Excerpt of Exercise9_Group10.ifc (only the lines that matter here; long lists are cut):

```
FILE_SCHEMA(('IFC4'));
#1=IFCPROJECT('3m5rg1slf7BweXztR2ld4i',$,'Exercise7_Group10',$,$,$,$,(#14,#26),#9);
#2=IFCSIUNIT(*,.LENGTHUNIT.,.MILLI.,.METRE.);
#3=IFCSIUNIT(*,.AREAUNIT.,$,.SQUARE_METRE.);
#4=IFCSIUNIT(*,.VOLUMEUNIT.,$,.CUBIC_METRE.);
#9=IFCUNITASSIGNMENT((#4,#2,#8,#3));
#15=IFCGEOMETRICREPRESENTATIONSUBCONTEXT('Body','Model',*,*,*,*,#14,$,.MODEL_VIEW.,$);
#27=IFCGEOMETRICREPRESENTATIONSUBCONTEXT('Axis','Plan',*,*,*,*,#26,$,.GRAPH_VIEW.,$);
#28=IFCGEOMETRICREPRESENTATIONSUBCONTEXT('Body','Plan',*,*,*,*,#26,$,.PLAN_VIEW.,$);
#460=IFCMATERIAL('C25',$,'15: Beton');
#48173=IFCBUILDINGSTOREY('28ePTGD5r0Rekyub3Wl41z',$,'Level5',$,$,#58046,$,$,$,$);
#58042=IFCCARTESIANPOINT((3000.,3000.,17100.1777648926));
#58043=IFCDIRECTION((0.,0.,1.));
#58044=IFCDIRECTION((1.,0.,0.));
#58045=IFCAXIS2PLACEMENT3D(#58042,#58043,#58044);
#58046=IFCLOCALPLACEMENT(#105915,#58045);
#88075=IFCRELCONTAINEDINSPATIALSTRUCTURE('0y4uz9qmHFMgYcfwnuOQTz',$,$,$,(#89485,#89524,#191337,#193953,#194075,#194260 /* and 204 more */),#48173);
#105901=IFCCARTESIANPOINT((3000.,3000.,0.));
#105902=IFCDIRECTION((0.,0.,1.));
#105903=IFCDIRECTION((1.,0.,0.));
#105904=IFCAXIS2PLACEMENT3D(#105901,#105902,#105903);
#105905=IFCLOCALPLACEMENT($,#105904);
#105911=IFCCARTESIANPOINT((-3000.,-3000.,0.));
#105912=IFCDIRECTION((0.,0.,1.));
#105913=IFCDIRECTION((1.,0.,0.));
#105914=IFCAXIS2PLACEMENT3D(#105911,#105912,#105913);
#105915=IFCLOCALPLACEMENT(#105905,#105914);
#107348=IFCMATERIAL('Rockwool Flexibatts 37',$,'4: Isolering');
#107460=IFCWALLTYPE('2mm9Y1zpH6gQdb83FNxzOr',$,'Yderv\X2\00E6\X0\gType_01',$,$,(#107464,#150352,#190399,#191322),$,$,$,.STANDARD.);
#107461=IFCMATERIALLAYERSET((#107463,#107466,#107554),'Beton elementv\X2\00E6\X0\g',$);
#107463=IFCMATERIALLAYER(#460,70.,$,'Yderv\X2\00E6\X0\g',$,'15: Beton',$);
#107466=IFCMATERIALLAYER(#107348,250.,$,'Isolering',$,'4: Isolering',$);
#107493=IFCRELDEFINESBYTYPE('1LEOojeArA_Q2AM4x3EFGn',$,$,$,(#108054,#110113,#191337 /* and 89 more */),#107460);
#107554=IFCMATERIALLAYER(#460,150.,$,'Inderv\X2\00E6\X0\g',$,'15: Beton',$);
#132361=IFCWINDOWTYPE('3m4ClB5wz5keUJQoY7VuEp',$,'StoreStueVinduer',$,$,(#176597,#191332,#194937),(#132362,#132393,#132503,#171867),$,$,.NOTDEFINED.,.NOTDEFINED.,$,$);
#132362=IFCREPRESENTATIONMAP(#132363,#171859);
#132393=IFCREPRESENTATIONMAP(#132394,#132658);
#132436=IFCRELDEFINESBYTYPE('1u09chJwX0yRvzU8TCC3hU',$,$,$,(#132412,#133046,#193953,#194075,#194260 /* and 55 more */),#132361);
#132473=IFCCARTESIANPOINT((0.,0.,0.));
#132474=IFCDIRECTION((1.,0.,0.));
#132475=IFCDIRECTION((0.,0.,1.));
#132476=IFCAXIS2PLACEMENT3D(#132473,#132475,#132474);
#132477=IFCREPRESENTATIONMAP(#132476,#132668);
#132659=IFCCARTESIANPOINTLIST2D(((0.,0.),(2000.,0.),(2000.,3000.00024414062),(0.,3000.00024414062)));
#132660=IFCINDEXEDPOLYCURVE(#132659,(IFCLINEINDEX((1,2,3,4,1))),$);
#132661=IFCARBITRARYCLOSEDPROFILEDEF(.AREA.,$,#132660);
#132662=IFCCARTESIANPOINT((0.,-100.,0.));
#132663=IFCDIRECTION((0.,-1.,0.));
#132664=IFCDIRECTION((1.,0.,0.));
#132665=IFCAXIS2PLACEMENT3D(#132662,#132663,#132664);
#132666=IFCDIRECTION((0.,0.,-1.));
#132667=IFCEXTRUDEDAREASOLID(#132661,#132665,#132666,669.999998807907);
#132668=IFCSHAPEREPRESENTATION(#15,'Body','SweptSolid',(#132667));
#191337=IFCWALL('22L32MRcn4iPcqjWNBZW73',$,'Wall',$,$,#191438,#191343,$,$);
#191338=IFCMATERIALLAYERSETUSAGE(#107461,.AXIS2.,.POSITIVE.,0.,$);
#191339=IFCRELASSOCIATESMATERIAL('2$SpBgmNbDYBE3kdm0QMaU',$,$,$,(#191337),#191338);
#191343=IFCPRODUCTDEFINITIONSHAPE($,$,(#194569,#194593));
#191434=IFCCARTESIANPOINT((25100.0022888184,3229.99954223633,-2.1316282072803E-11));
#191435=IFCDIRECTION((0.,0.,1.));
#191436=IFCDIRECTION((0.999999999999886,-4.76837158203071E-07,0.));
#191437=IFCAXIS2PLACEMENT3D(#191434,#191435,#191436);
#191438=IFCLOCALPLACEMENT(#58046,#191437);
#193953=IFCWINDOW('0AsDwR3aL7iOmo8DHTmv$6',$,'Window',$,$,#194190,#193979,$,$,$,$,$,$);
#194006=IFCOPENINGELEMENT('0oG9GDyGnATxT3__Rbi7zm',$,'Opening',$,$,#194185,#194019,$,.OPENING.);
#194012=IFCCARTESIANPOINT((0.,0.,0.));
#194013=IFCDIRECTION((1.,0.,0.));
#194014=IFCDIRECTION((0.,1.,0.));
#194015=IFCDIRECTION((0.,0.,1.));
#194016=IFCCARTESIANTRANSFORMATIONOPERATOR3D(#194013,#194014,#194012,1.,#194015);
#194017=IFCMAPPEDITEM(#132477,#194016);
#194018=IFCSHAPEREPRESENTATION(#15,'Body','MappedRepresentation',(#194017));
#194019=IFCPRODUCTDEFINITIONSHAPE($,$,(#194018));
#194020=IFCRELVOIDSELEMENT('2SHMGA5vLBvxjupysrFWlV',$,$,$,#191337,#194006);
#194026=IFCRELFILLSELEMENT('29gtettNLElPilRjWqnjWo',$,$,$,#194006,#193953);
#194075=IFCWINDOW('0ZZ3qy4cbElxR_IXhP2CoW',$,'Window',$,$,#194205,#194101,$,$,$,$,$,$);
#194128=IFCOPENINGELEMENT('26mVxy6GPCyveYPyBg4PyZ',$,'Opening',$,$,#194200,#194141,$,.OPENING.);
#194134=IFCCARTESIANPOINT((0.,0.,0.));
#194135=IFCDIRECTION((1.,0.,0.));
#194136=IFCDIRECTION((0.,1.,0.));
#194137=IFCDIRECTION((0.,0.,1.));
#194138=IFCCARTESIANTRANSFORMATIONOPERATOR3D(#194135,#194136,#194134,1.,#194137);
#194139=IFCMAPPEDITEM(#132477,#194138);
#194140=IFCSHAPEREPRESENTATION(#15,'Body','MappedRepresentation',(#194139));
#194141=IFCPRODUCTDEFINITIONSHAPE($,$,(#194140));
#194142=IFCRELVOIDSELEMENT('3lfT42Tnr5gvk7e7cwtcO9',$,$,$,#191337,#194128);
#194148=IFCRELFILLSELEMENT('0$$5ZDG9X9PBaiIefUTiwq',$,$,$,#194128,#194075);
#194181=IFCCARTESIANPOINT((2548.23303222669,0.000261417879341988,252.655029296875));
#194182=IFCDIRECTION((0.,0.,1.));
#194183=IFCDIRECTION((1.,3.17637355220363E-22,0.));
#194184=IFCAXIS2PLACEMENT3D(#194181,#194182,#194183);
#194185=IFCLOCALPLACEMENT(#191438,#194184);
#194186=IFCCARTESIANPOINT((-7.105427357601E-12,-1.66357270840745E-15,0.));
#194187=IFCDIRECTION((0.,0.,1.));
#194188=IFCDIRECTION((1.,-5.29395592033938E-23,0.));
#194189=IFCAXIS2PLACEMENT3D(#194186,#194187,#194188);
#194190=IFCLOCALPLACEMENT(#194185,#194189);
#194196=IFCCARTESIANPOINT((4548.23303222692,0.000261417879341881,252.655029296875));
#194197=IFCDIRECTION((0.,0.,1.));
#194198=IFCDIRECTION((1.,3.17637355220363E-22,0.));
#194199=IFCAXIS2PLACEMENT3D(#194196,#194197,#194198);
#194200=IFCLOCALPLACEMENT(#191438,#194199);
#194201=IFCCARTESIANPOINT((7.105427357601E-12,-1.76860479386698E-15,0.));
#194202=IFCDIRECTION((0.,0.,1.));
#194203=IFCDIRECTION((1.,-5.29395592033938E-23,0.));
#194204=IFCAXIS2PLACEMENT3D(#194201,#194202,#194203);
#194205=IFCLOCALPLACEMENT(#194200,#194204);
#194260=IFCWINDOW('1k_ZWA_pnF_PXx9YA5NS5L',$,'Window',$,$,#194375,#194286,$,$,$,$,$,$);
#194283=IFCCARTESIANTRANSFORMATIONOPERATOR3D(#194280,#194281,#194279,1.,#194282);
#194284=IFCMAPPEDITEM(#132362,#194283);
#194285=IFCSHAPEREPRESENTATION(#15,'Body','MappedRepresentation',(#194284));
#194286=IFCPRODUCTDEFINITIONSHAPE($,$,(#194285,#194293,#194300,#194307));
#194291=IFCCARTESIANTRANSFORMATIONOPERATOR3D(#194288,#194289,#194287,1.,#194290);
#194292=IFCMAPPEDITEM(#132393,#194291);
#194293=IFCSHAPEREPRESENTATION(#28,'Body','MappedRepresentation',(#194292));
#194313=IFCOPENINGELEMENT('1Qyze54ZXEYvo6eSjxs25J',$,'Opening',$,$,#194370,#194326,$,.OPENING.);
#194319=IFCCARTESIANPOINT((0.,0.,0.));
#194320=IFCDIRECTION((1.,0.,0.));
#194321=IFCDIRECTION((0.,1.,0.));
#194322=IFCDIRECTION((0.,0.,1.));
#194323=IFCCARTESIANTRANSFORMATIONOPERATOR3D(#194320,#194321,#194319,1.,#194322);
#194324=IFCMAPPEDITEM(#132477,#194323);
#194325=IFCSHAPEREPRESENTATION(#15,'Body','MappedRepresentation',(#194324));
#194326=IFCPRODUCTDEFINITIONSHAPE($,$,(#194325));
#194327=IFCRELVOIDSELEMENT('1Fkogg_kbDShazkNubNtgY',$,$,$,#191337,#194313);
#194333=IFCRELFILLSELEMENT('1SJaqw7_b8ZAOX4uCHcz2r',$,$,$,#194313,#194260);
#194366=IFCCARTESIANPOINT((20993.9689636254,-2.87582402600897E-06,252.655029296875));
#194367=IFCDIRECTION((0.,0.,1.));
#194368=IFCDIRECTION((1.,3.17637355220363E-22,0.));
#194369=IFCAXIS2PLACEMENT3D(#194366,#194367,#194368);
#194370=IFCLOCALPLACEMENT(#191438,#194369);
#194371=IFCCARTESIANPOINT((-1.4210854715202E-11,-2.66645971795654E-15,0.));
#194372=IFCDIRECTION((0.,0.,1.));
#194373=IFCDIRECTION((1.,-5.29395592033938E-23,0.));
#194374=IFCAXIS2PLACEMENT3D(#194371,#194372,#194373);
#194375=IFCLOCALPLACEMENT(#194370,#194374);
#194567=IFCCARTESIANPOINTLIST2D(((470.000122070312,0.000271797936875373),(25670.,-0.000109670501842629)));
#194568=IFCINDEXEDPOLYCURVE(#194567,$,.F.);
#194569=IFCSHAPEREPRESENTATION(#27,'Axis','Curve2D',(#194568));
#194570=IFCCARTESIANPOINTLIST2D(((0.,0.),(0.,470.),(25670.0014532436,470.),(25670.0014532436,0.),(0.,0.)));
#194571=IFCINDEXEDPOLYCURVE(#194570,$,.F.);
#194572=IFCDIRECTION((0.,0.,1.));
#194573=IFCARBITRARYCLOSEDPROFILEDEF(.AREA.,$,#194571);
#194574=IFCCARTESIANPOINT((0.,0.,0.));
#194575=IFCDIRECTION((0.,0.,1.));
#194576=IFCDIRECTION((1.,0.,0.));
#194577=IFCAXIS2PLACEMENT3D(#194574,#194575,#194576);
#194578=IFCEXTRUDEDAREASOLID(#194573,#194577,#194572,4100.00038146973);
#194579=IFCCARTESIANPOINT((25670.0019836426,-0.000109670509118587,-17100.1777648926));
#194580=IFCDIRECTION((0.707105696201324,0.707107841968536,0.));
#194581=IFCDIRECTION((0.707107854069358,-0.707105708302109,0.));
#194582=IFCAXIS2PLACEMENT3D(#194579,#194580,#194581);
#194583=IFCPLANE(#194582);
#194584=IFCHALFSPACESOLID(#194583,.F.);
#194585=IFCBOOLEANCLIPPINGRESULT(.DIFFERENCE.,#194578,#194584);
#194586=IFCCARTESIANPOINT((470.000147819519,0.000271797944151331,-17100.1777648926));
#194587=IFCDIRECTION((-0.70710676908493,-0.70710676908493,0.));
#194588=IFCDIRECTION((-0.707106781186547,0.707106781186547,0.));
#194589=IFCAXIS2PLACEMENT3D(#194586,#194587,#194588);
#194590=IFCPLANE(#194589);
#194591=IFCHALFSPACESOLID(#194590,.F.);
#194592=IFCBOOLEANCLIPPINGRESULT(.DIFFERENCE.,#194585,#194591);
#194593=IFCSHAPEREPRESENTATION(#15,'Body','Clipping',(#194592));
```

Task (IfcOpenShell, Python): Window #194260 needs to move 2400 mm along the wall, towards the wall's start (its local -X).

```python
import ifcopenshell
import ifcopenshell.api.geometry
import ifcopenshell.util.placement
import ifcopenshell.util.unit

model = ifcopenshell.open("Exercise9_Group10.ifc")
unit_scale = ifcopenshell.util.unit.calculate_unit_scale(model)

window = model.by_guid("1k_ZWA_pnF_PXx9YA5NS5L")
opening = window.FillsVoids[0].RelatingOpeningElement
wall = opening.VoidsElements[0].RelatingBuildingElement

wall_matrix = ifcopenshell.util.placement.get_local_placement(wall.ObjectPlacement)
shift = wall_matrix[:3, 0] * -2.4 / unit_scale
before = ifcopenshell.util.placement.get_local_placement(window.ObjectPlacement)[:3, 3].copy()

# The window is placed relative to its opening, so it follows when the opening moves.
matrix = ifcopenshell.util.placement.get_local_placement(opening.ObjectPlacement)
matrix[:3, 3] += shift
ifcopenshell.api.geometry.edit_object_placement(
    model, product=opening, matrix=matrix, is_si=False, should_transform_children=True
)

after = ifcopenshell.util.placement.get_local_placement(window.ObjectPlacement)[:3, 3]
print("window moved by", (after - before).round(3) + 0.0)

model.write("Exercise9_Group10_edited.ifc")
```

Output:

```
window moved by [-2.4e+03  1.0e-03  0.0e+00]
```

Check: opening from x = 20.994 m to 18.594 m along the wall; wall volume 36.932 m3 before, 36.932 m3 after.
